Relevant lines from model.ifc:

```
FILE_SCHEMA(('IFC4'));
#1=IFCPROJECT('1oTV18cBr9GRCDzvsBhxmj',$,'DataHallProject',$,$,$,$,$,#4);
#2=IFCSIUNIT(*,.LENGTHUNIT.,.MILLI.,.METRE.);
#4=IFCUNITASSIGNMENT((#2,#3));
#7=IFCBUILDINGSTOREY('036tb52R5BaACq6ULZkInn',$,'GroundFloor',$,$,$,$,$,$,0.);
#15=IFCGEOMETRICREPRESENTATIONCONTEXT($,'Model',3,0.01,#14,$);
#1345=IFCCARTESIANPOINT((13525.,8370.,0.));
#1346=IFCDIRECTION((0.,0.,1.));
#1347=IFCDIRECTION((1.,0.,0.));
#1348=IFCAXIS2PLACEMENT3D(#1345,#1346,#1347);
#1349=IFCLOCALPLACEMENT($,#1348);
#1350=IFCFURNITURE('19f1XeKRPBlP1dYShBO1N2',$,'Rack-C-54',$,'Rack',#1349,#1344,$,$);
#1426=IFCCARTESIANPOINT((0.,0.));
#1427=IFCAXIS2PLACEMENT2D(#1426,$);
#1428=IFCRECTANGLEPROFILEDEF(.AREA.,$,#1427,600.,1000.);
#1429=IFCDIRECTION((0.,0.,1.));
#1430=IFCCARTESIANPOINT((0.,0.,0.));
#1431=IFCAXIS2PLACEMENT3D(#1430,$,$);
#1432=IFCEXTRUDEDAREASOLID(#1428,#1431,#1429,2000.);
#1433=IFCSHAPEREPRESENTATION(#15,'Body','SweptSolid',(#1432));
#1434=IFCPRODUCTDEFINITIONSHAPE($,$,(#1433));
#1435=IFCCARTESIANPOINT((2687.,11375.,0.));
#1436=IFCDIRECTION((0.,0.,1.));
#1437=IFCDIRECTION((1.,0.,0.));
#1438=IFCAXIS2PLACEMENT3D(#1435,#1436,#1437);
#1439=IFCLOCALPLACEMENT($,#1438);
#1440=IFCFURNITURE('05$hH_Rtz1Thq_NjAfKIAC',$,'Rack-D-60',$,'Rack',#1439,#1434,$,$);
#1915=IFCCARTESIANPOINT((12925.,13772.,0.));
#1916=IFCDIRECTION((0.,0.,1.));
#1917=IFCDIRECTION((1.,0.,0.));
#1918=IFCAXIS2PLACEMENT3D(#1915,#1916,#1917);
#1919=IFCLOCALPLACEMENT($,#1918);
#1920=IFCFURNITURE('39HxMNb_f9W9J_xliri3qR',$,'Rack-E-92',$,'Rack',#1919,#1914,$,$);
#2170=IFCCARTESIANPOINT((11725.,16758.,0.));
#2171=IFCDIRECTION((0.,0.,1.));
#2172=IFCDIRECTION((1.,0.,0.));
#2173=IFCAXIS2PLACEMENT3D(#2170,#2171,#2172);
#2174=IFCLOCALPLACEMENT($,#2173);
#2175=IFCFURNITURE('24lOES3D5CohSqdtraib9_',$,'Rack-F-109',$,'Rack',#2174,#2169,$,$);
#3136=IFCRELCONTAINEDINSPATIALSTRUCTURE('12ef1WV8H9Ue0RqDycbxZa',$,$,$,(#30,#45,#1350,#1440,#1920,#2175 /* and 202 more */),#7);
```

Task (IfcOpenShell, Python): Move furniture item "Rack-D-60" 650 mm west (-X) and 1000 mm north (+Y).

```python
import ifcopenshell
import ifcopenshell.api.geometry
import ifcopenshell.util.placement

model = ifcopenshell.open("model.ifc")

item = model.by_id(1440)
matrix = ifcopenshell.util.placement.get_local_placement(item.ObjectPlacement)
matrix[0, 3] -= 650.0
matrix[1, 3] += 1000.0
ifcopenshell.api.geometry.edit_object_placement(model, product=item, matrix=matrix, is_si=False)

print(ifcopenshell.util.placement.get_local_placement(item.ObjectPlacement).round(3) + 0.0)

model.write("model_rev.ifc")
```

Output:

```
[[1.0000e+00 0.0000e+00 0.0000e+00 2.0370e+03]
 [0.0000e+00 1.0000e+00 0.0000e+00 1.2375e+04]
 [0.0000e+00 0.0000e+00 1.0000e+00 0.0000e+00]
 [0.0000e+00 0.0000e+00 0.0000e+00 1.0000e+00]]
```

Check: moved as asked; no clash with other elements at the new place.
